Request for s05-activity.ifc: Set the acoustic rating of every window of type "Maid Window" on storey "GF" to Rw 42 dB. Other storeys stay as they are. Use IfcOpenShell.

First a look at what the model holds.

```python
import ifcopenshell
import ifcopenshell.util.element

model = ifcopenshell.open("s05-activity.ifc")
print(model.schema)
storey = next(s for s in model.by_type("IfcBuildingStorey") if s.Name == "GF")
windows = [e for e in ifcopenshell.util.element.get_decomposition(storey) if e.is_a("IfcWindow")]
seen = {}
for e in windows:
    element_type = ifcopenshell.util.element.get_type(e)
    key = (element_type.Name if element_type != e and element_type else None, ifcopenshell.util.element.get_pset(e, "Pset_WindowCommon", "AcousticRating"))
    seen[key] = seen.get(key, 0) + 1
for (name, value), count in sorted(seen.items(), key=str):
    print(count, "x", name, "|", value)
```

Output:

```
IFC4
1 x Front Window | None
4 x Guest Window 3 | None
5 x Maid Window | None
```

```python
import ifcopenshell
import ifcopenshell.api.pset
import ifcopenshell.util.element

model = ifcopenshell.open("s05-activity.ifc")

storey = next(s for s in model.by_type("IfcBuildingStorey") if s.Name == "GF")
windows = [e for e in ifcopenshell.util.element.get_decomposition(storey) if e.is_a("IfcWindow")]

count = 0
for e in windows:
    element_type = ifcopenshell.util.element.get_type(e)
    if element_type in (None, e) or element_type.Name != "Maid Window":
        continue
    # add_pset returns the element's existing set when there is one.
    pset = ifcopenshell.api.pset.add_pset(model, product=e, name="Pset_WindowCommon")
    ifcopenshell.api.pset.edit_pset(model, pset=pset, properties={"AcousticRating": "Rw 42 dB"})
    count += 1

print(count, "windows updated")

model.write("s05-activity_rev.ifc")
```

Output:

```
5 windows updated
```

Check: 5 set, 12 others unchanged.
